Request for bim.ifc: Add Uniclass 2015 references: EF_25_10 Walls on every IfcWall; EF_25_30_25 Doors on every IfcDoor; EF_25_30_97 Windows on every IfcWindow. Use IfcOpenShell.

First a look at what the model holds.

```python
import ifcopenshell

model = ifcopenshell.open("bim.ifc")
print(model.schema)
print("classifications:", [c.Name for c in model.by_type("IfcClassification")])
for ifc_class in ("IfcDoor", "IfcRoof", "IfcStair", "IfcWall", "IfcWindow"):
    print(ifc_class, len(model.by_type(ifc_class)))
```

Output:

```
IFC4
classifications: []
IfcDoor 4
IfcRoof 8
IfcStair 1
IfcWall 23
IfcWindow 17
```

```python
import ifcopenshell
import ifcopenshell.api.classification

model = ifcopenshell.open("bim.ifc")

system = ifcopenshell.api.classification.add_classification(model, classification="Uniclass 2015")

codes = {
    "IfcWall": ("EF_25_10", "Walls"),
    "IfcDoor": ("EF_25_30_25", "Doors"),
    "IfcWindow": ("EF_25_30_97", "Windows"),
}
for ifc_class, (code, name) in codes.items():
    products = model.by_type(ifc_class)
    ifcopenshell.api.classification.add_reference(
        model, products=products, classification=system, identification=code, name=name
    )
    print(code, len(products))

model.write("bim_v2.ifc")
```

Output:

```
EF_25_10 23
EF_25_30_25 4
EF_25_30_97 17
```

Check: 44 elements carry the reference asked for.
